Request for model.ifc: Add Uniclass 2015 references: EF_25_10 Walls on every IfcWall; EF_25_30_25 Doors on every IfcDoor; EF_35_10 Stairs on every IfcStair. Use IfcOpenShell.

First a look at what the model holds.

```python
import ifcopenshell

model = ifcopenshell.open("model.ifc")
print(model.schema)
print("classifications:", [c.Name for c in model.by_type("IfcClassification")])
for ifc_class in ("IfcDoor", "IfcRoof", "IfcStair", "IfcWall", "IfcWindow"):
    print(ifc_class, len(model.by_type(ifc_class)))
```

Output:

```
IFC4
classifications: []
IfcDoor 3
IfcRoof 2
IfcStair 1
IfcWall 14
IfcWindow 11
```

```python
import ifcopenshell
import ifcopenshell.api.classification

model = ifcopenshell.open("model.ifc")

system = ifcopenshell.api.classification.add_classification(model, classification="Uniclass 2015")

codes = {
    "IfcWall": ("EF_25_10", "Walls"),
    "IfcDoor": ("EF_25_30_25", "Doors"),
    "IfcStair": ("EF_35_10", "Stairs"),
}
for ifc_class, (code, name) in codes.items():
    products = model.by_type(ifc_class)
    ifcopenshell.api.classification.add_reference(
        model, products=products, classification=system, identification=code, name=name
    )
    print(code, len(products))

model.write("model_edited.ifc")
```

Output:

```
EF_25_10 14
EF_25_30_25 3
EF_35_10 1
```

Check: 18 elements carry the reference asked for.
